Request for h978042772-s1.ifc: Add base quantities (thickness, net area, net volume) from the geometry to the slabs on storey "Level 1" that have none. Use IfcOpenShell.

First a look at what the model holds.

```python
import ifcopenshell
import ifcopenshell.util.element
import ifcopenshell.util.unit

model = ifcopenshell.open("h978042772-s1.ifc")
print(model.schema)
for unit_type in ("LENGTHUNIT", "AREAUNIT", "VOLUMEUNIT"):
    print(unit_type, ifcopenshell.util.unit.calculate_unit_scale(model, unit_type))
storey = next(s for s in model.by_type("IfcBuildingStorey") if s.Name == "Level 1")
slabs = [e for e in ifcopenshell.util.element.get_decomposition(storey) if e.is_a("IfcSlab")]
for e in sorted(slabs, key=lambda e: e.id()):
    print(e.id(), e.is_a(), e.Name, list(ifcopenshell.util.element.get_psets(e, qtos_only=True)), sep=" | ")
```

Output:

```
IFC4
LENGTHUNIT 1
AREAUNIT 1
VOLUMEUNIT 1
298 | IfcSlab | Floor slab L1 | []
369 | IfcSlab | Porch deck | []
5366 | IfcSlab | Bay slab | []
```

```python
import ifcopenshell
import ifcopenshell.api.pset
import ifcopenshell.geom
import ifcopenshell.util.element
import ifcopenshell.util.shape
import ifcopenshell.util.unit

model = ifcopenshell.open("h978042772-s1.ifc")
unit_scale = ifcopenshell.util.unit.calculate_unit_scale(model)
area_scale = ifcopenshell.util.unit.calculate_unit_scale(model, "AREAUNIT")
volume_scale = ifcopenshell.util.unit.calculate_unit_scale(model, "VOLUMEUNIT")
settings = ifcopenshell.geom.settings()

storey = next(s for s in model.by_type("IfcBuildingStorey") if s.Name == "Level 1")
slabs = [e for e in ifcopenshell.util.element.get_decomposition(storey) if e.is_a("IfcSlab")]

for e in sorted(slabs, key=lambda e: e.id()):
    if ifcopenshell.util.element.get_psets(e, qtos_only=True, should_inherit=False):
        continue
    # Geometry comes back in metres, in the element's own axes.
    shape = ifcopenshell.geom.create_shape(settings, e)
    values = {
        "Width": ifcopenshell.util.shape.get_z(shape.geometry) / unit_scale,
        "NetArea": ifcopenshell.util.shape.get_footprint_area(shape.geometry) / area_scale,
        "NetVolume": ifcopenshell.util.shape.get_volume(shape.geometry) / volume_scale,
    }
    qto = ifcopenshell.api.pset.add_qto(model, product=e, name="Qto_SlabBaseQuantities")
    ifcopenshell.api.pset.edit_qto(model, qto=qto, properties=values)
    print(e.id(), {k: round(v, 3) for k, v in values.items()})

model.write("h978042772-s1_updated.ifc")
```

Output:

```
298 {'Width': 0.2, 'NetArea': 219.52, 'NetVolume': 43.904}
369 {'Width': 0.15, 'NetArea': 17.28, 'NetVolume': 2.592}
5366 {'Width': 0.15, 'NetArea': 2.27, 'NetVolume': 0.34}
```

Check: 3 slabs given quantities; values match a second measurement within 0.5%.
